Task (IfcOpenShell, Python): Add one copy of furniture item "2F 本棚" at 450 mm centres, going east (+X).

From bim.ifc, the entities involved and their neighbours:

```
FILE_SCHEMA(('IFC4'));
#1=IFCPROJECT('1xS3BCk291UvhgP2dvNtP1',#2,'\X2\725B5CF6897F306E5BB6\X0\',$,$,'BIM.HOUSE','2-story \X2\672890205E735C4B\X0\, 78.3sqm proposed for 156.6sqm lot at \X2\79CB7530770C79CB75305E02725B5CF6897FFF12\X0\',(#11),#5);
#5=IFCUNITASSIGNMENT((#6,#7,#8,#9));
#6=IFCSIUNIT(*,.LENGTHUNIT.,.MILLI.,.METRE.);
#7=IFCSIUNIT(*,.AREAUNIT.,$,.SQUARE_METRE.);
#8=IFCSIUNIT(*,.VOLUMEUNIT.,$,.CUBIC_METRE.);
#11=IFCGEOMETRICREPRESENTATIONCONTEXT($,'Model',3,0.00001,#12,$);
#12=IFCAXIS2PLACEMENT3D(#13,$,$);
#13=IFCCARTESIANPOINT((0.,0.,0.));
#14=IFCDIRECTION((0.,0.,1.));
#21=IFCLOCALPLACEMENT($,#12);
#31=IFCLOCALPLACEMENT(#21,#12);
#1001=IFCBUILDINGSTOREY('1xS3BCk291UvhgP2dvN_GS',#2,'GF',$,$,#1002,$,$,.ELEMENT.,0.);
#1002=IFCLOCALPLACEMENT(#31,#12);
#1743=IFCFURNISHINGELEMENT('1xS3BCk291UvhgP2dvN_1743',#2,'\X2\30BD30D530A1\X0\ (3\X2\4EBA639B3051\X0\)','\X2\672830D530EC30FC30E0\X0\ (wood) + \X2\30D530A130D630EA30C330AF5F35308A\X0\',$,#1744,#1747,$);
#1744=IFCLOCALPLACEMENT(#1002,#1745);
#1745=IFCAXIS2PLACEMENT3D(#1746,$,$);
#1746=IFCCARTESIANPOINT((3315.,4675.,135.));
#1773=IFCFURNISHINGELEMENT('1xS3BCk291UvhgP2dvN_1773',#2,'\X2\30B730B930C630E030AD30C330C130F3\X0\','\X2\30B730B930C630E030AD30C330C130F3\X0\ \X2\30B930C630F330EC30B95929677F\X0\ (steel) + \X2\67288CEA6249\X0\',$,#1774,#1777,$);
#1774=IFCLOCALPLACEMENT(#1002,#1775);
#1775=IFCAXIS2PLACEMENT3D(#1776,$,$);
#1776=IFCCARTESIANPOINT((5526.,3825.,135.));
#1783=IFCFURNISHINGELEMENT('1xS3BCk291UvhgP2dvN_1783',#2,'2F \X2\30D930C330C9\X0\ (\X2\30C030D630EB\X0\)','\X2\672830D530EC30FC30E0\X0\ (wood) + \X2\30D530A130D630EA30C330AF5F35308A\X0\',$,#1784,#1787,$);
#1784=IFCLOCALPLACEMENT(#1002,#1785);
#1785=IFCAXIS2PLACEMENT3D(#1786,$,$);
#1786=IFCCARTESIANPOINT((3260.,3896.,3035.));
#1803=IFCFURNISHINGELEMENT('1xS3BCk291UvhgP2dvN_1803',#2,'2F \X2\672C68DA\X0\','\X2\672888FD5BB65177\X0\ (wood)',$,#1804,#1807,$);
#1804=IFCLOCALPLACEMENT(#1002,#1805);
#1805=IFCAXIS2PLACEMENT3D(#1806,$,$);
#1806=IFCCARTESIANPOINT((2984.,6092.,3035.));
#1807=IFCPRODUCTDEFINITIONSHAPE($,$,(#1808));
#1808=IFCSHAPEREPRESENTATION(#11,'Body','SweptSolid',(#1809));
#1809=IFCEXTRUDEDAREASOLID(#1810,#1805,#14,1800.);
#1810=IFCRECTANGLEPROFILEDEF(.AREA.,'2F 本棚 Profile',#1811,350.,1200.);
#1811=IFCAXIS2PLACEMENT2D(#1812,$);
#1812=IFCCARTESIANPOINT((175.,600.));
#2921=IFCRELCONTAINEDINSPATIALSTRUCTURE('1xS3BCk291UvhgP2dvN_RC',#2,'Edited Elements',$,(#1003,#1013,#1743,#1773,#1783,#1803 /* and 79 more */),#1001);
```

```python
import numpy as np
import ifcopenshell
import ifcopenshell.api.geometry
import ifcopenshell.api.root
import ifcopenshell.util.element
import ifcopenshell.util.placement
import ifcopenshell.util.unit

model = ifcopenshell.open("bim.ifc")
unit_scale = ifcopenshell.util.unit.calculate_unit_scale(model)


def reuse_history(source, copy):
    """copy_class also copies each property set's owner history, people and application; keep the originals."""
    for rel in copy.IsDefinedBy:
        if rel.is_a("IfcRelDefinesByProperties") and (history := rel.RelatingPropertyDefinition.OwnerHistory):
            rel.RelatingPropertyDefinition.OwnerHistory = source.OwnerHistory
            ifcopenshell.util.element.remove_deep2(model, history)


source = model.by_id(1803)
base = ifcopenshell.util.placement.get_local_placement(source.ObjectPlacement)
step = np.array([1.0, 0.0, 0.0]) * 0.45 / unit_scale

for i in range(1, 2):
    copy = ifcopenshell.api.root.copy_class(model, product=source)
    copy.Representation = ifcopenshell.util.element.copy_deep(
        model, source.Representation, exclude=["IfcGeometricRepresentationContext", "IfcRepresentationMap"]
    )
    reuse_history(source, copy)
    matrix = base.copy()
    matrix[:3, 3] += i * step
    print("added at", matrix[:3, 3].round(3) + 0.0)
    ifcopenshell.api.geometry.edit_object_placement(model, product=copy, matrix=matrix, is_si=False)

model.write("bim_edited.ifc")
```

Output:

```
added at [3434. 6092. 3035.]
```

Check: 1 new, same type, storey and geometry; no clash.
